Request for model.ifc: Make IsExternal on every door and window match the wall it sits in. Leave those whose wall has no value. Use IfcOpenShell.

First a look at what the model holds.

```python
import ifcopenshell
import ifcopenshell.util.element

model = ifcopenshell.open("model.ifc")
print(model.schema)
seen = {}
for e in model.by_type("IfcDoor") + model.by_type("IfcWindow"):
    if not e.FillsVoids:
        continue
    host = e.FillsVoids[0].RelatingOpeningElement.VoidsElements[0].RelatingBuildingElement
    own = ifcopenshell.util.element.get_pset(e, f"Pset_{e.is_a()[3:].removesuffix('StandardCase')}Common", "IsExternal")
    wall = ifcopenshell.util.element.get_pset(host, "Pset_WallCommon", "IsExternal")
    seen[e.is_a(), own, wall] = seen.get((e.is_a(), own, wall), 0) + 1
for (cls, own, wall), count in sorted(seen.items(), key=str):
    print(count, cls, "IsExternal:", own, "| host wall:", wall)
```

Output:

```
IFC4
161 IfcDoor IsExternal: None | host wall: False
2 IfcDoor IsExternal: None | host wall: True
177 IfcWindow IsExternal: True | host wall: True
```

```python
import ifcopenshell
import ifcopenshell.api.pset
import ifcopenshell.util.element

model = ifcopenshell.open("model.ifc")

count = 0
for ifc_class, pset_name in (("IfcDoor", "Pset_DoorCommon"), ("IfcWindow", "Pset_WindowCommon")):
    for e in model.by_type(ifc_class):
        if not e.FillsVoids:
            continue
        host = e.FillsVoids[0].RelatingOpeningElement.VoidsElements[0].RelatingBuildingElement
        external = ifcopenshell.util.element.get_pset(host, "Pset_WallCommon", "IsExternal")
        if external is None or ifcopenshell.util.element.get_pset(e, pset_name, "IsExternal") == external:
            continue
        found = ifcopenshell.util.element.get_pset(e, pset_name, should_inherit=False)
        if found:
            pset = model.by_id(found["id"])
            if len(ifcopenshell.util.element.get_elements_by_pset(pset)) > 1:
                pset = ifcopenshell.api.pset.unshare_pset(model, products=[e], pset=pset)[0]
        else:
            pset = ifcopenshell.api.pset.add_pset(model, product=e, name=pset_name)
        ifcopenshell.api.pset.edit_pset(model, pset=pset, properties={"IsExternal": external})
        count += 1

print(count, "updated")

model.write("model_updated.ifc")
```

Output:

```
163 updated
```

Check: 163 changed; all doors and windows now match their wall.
